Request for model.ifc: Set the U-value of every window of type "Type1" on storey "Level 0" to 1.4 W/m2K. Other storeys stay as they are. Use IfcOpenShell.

First a look at what the model holds.

```python
import ifcopenshell
import ifcopenshell.util.element

model = ifcopenshell.open("model.ifc")
print(model.schema)
storey = next(s for s in model.by_type("IfcBuildingStorey") if s.Name == "Level 0")
windows = [e for e in ifcopenshell.util.element.get_decomposition(storey) if e.is_a("IfcWindow")]
seen = {}
for e in windows:
    element_type = ifcopenshell.util.element.get_type(e)
    key = (element_type.Name if element_type != e and element_type else None, ifcopenshell.util.element.get_pset(e, "Pset_WindowCommon", "ThermalTransmittance"))
    seen[key] = seen.get(key, 0) + 1
for (name, value), count in sorted(seen.items(), key=str):
    print(count, "x", name, "|", value)
```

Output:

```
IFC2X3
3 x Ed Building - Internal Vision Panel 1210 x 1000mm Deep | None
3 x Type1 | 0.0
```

```python
import ifcopenshell
import ifcopenshell.api.pset
import ifcopenshell.util.element

model = ifcopenshell.open("model.ifc")

storey = next(s for s in model.by_type("IfcBuildingStorey") if s.Name == "Level 0")
windows = [e for e in ifcopenshell.util.element.get_decomposition(storey) if e.is_a("IfcWindow")]

count = 0
for e in windows:
    element_type = ifcopenshell.util.element.get_type(e)
    if element_type in (None, e) or element_type.Name != "Type1":
        continue
    # add_pset returns the element's existing set when there is one.
    pset = ifcopenshell.api.pset.add_pset(model, product=e, name="Pset_WindowCommon")
    ifcopenshell.api.pset.edit_pset(model, pset=pset, properties={"ThermalTransmittance": 1.4})
    count += 1

print(count, "windows updated")

model.write("model-out.ifc")
```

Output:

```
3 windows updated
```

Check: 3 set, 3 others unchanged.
